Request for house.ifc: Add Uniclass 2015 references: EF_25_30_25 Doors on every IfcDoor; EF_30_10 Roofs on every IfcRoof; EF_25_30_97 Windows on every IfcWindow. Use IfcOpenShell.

First a look at what the model holds.

```python
import ifcopenshell

model = ifcopenshell.open("house.ifc")
print(model.schema)
print("classifications:", [c.Name for c in model.by_type("IfcClassification")])
for ifc_class in ("IfcDoor", "IfcRoof", "IfcStair", "IfcWall", "IfcWindow"):
    print(ifc_class, len(model.by_type(ifc_class)))
```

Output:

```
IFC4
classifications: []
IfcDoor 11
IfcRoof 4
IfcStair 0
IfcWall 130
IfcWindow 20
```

```python
import ifcopenshell
import ifcopenshell.api.classification

model = ifcopenshell.open("house.ifc")

system = ifcopenshell.api.classification.add_classification(model, classification="Uniclass 2015")

codes = {
    "IfcDoor": ("EF_25_30_25", "Doors"),
    "IfcRoof": ("EF_30_10", "Roofs"),
    "IfcWindow": ("EF_25_30_97", "Windows"),
}
for ifc_class, (code, name) in codes.items():
    products = model.by_type(ifc_class)
    ifcopenshell.api.classification.add_reference(
        model, products=products, classification=system, identification=code, name=name
    )
    print(code, len(products))

model.write("house_v2.ifc")
```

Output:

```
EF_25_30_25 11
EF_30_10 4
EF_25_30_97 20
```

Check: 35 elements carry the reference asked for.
